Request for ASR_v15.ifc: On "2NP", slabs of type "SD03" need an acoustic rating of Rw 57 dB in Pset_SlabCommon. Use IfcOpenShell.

First a look at what the model holds.

```python
import ifcopenshell
import ifcopenshell.util.element

model = ifcopenshell.open("ASR_v15.ifc")
print(model.schema)
storey = next(s for s in model.by_type("IfcBuildingStorey") if s.Name == "2NP")
slabs = [e for e in ifcopenshell.util.element.get_decomposition(storey) if e.is_a("IfcSlab")]
seen = {}
for e in slabs:
    element_type = ifcopenshell.util.element.get_type(e)
    key = (element_type.Name if element_type != e and element_type else None, ifcopenshell.util.element.get_pset(e, "Pset_SlabCommon", "AcousticRating"))
    seen[key] = seen.get(key, 0) + 1
for (name, value), count in sorted(seen.items(), key=str):
    print(count, "x", name, "|", value)
```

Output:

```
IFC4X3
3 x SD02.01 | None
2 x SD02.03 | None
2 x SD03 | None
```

```python
import ifcopenshell
import ifcopenshell.api.pset
import ifcopenshell.util.element

model = ifcopenshell.open("ASR_v15.ifc")

storey = next(s for s in model.by_type("IfcBuildingStorey") if s.Name == "2NP")
slabs = [e for e in ifcopenshell.util.element.get_decomposition(storey) if e.is_a("IfcSlab")]

count = 0
for e in slabs:
    element_type = ifcopenshell.util.element.get_type(e)
    if element_type in (None, e) or element_type.Name != "SD03":
        continue
    # add_pset returns the element's existing set when there is one.
    pset = ifcopenshell.api.pset.add_pset(model, product=e, name="Pset_SlabCommon")
    ifcopenshell.api.pset.edit_pset(model, pset=pset, properties={"AcousticRating": "Rw 57 dB"})
    count += 1

print(count, "slabs updated")

model.write("ASR_v15-out.ifc")
```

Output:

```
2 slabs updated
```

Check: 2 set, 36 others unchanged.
